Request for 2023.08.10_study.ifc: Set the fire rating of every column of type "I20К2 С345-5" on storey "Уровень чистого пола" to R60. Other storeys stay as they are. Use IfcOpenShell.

First a look at what the model holds.

```python
import ifcopenshell
import ifcopenshell.util.element

model = ifcopenshell.open("2023.08.10_study.ifc")
print(model.schema)
storey = next(s for s in model.by_type("IfcBuildingStorey") if s.Name == "Уровень чистого пола")
columns = [e for e in ifcopenshell.util.element.get_decomposition(storey) if e.is_a("IfcColumn")]
seen = {}
for e in columns:
    element_type = ifcopenshell.util.element.get_type(e)
    key = (element_type.Name if element_type != e and element_type else None, ifcopenshell.util.element.get_pset(e, "Pset_ColumnCommon", "FireRating"))
    seen[key] = seen.get(key, 0) + 1
for (name, value), count in sorted(seen.items(), key=str):
    print(count, "x", name, "|", value)
```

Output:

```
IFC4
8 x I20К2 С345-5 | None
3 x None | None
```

```python
import ifcopenshell
import ifcopenshell.api.pset
import ifcopenshell.util.element

model = ifcopenshell.open("2023.08.10_study.ifc")

storey = next(s for s in model.by_type("IfcBuildingStorey") if s.Name == "Уровень чистого пола")
columns = [e for e in ifcopenshell.util.element.get_decomposition(storey) if e.is_a("IfcColumn")]

count = 0
for e in columns:
    element_type = ifcopenshell.util.element.get_type(e)
    if element_type in (None, e) or element_type.Name != "I20К2 С345-5":
        continue
    # add_pset returns the element's existing set when there is one.
    pset = ifcopenshell.api.pset.add_pset(model, product=e, name="Pset_ColumnCommon")
    ifcopenshell.api.pset.edit_pset(model, pset=pset, properties={"FireRating": "R60"})
    count += 1

print(count, "columns updated")

model.write("2023.08.10_study-out.ifc")
```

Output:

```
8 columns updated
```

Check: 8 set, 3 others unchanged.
